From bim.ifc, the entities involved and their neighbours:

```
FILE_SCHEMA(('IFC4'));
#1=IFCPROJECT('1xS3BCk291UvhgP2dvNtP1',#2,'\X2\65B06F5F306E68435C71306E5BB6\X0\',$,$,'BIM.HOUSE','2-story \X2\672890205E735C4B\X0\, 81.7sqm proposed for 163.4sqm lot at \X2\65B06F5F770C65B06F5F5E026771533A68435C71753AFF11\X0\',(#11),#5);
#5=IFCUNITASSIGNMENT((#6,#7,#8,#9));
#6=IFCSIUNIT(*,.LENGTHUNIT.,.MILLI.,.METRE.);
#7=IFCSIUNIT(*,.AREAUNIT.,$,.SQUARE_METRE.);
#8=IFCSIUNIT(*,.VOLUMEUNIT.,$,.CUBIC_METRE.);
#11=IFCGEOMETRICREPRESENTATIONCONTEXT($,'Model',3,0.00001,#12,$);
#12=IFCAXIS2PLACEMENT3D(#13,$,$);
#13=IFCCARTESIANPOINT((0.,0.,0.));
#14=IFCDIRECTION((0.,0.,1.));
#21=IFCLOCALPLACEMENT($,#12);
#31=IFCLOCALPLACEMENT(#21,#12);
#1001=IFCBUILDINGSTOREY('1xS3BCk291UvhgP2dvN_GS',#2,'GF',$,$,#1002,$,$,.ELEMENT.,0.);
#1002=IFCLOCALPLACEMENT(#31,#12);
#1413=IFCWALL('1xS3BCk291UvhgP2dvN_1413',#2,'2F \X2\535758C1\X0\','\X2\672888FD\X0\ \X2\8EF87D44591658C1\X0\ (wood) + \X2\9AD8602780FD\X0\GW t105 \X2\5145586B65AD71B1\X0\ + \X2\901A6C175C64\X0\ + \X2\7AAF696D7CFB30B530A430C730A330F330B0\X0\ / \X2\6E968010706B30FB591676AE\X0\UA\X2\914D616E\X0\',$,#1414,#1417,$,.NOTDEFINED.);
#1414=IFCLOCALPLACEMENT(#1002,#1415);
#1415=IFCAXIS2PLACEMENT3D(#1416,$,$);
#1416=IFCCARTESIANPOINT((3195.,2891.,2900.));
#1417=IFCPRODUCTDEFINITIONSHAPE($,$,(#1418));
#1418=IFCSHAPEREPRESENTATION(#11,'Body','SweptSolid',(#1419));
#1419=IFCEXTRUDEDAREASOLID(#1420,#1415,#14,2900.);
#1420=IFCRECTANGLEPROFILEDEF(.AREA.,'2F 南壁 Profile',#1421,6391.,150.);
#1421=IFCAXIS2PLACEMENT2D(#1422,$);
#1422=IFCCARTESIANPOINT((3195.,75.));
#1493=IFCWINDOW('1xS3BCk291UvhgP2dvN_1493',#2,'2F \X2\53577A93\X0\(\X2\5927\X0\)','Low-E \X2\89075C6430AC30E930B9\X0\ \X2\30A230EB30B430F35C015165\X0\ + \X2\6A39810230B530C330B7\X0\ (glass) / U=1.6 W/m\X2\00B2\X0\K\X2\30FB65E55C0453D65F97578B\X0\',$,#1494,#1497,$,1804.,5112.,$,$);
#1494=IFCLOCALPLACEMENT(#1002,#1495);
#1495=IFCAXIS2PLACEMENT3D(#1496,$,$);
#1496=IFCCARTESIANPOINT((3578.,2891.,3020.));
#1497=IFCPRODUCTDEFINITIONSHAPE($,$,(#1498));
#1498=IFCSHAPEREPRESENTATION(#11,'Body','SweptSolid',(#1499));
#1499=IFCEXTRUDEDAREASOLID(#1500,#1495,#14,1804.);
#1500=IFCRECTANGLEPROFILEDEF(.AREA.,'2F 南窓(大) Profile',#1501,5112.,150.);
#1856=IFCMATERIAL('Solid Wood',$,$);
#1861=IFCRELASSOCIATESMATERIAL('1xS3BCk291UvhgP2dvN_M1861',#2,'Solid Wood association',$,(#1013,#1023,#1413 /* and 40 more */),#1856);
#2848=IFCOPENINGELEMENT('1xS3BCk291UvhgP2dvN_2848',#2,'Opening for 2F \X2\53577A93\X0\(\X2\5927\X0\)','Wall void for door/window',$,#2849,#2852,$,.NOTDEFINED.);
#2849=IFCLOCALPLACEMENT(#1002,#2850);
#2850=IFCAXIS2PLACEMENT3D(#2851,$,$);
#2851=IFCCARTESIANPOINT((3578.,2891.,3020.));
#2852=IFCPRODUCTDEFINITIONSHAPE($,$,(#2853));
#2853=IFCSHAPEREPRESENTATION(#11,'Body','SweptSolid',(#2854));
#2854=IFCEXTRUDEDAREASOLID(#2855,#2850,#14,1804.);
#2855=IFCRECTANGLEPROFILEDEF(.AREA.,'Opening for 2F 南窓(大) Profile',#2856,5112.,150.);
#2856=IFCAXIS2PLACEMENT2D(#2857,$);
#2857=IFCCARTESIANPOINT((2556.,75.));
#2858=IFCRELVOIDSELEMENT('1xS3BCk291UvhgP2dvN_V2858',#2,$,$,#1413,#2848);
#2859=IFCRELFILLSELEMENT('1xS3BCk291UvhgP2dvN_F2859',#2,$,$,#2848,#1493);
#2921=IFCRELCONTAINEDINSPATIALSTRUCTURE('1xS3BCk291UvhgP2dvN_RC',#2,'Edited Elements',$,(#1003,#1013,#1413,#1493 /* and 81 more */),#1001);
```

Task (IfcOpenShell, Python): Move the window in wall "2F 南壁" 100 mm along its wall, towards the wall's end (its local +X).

```python
import ifcopenshell
import ifcopenshell.api.geometry
import ifcopenshell.util.placement

model = ifcopenshell.open("bim.ifc")

window = model.by_id(1493)
opening = window.FillsVoids[0].RelatingOpeningElement
wall = opening.VoidsElements[0].RelatingBuildingElement

wall_matrix = ifcopenshell.util.placement.get_local_placement(wall.ObjectPlacement)
shift = wall_matrix[:3, 0] * 100.0
before = ifcopenshell.util.placement.get_local_placement(window.ObjectPlacement)[:3, 3].copy()

# The window is not placed relative to its opening, so move both.
for product in (opening, window):
    matrix = ifcopenshell.util.placement.get_local_placement(product.ObjectPlacement)
    matrix[:3, 3] += shift
    ifcopenshell.api.geometry.edit_object_placement(model, product=product, matrix=matrix, is_si=False)

after = ifcopenshell.util.placement.get_local_placement(window.ObjectPlacement)[:3, 3]
print("window moved by", (after - before).round(3) + 0.0)

model.write("bim-out.ifc")
```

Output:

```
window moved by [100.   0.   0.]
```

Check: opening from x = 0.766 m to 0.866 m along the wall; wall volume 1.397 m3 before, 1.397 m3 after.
